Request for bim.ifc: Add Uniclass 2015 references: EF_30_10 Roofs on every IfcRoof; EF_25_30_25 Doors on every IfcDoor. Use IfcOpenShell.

First a look at what the model holds.

```python
import ifcopenshell

model = ifcopenshell.open("bim.ifc")
print(model.schema)
print("classifications:", [c.Name for c in model.by_type("IfcClassification")])
for ifc_class in ("IfcDoor", "IfcRoof", "IfcStair", "IfcWall", "IfcWindow"):
    print(ifc_class, len(model.by_type(ifc_class)))
```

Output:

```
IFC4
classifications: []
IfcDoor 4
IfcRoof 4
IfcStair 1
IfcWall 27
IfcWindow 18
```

```python
import ifcopenshell
import ifcopenshell.api.classification

model = ifcopenshell.open("bim.ifc")

system = ifcopenshell.api.classification.add_classification(model, classification="Uniclass 2015")

codes = {
    "IfcRoof": ("EF_30_10", "Roofs"),
    "IfcDoor": ("EF_25_30_25", "Doors"),
}
for ifc_class, (code, name) in codes.items():
    products = model.by_type(ifc_class)
    ifcopenshell.api.classification.add_reference(
        model, products=products, classification=system, identification=code, name=name
    )
    print(code, len(products))

model.write("bim_updated.ifc")
```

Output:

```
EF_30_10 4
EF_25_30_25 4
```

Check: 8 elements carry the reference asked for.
